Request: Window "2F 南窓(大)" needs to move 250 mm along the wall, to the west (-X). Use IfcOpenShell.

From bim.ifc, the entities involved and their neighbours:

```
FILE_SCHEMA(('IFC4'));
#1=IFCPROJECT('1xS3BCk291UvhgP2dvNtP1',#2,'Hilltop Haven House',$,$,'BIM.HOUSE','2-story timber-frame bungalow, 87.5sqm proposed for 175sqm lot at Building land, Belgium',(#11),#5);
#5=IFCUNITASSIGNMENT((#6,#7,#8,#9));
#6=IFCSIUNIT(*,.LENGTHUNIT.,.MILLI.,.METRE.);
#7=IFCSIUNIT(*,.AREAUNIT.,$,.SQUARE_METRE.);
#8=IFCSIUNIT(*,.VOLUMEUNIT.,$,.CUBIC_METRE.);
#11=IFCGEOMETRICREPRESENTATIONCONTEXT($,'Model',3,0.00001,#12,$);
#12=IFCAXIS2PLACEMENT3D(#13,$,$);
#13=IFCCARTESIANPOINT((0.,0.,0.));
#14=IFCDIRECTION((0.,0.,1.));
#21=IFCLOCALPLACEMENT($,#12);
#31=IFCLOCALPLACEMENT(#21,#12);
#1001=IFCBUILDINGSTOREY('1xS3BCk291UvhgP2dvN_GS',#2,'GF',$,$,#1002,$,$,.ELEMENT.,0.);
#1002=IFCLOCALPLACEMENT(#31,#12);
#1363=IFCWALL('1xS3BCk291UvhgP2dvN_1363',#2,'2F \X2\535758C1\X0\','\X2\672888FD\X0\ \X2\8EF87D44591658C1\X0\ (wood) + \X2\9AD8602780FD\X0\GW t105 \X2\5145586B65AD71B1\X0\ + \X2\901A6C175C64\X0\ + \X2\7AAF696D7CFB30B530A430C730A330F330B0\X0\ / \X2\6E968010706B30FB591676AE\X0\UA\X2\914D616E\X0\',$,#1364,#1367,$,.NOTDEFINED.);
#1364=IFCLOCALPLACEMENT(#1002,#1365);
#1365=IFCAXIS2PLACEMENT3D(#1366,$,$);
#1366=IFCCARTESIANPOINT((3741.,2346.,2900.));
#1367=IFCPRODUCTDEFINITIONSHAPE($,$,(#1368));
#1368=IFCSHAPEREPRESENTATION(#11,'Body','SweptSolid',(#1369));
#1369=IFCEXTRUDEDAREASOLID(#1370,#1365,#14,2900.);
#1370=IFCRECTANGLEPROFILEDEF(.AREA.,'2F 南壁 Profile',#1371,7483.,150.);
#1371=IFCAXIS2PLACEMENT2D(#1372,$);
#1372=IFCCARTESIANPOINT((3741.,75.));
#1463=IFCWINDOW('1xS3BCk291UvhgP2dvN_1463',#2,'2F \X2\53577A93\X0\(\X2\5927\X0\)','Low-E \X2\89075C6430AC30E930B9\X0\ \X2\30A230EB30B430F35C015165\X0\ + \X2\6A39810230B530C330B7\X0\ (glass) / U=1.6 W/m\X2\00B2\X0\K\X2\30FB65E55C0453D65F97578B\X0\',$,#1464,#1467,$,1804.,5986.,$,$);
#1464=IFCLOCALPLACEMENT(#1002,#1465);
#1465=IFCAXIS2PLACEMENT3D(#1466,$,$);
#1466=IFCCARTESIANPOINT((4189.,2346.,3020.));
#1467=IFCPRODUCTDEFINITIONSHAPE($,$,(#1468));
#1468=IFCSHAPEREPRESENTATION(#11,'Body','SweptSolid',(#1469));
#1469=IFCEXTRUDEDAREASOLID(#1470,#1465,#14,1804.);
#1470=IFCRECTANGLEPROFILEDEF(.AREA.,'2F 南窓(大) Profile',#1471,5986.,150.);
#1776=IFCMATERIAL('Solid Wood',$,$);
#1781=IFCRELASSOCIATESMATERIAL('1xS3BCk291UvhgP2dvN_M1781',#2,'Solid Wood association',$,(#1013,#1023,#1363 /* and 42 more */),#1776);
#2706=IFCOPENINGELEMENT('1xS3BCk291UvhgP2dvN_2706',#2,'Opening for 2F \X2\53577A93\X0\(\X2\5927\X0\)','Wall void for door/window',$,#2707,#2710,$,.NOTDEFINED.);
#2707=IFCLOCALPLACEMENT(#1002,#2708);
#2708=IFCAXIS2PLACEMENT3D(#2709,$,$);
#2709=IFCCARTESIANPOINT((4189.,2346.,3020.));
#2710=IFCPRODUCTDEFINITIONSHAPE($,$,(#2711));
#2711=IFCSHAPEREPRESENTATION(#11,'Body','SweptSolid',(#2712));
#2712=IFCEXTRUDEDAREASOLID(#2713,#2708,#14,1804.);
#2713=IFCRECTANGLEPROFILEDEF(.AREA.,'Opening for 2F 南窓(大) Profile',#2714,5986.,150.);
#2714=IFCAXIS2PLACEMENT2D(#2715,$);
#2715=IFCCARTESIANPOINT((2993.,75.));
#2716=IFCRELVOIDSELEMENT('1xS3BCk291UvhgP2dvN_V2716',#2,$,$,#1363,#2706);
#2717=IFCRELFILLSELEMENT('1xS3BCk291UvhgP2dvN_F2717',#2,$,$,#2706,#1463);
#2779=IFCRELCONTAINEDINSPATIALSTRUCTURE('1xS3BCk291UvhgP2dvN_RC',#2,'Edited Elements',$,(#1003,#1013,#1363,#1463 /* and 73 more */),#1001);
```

```python
import ifcopenshell
import ifcopenshell.api.geometry
import ifcopenshell.util.placement
import ifcopenshell.util.unit

model = ifcopenshell.open("bim.ifc")
unit_scale = ifcopenshell.util.unit.calculate_unit_scale(model)

window = model.by_guid("1xS3BCk291UvhgP2dvN_1463")
opening = window.FillsVoids[0].RelatingOpeningElement
wall = opening.VoidsElements[0].RelatingBuildingElement

wall_matrix = ifcopenshell.util.placement.get_local_placement(wall.ObjectPlacement)
shift = wall_matrix[:3, 0] * -0.25 / unit_scale
before = ifcopenshell.util.placement.get_local_placement(window.ObjectPlacement)[:3, 3].copy()

# The window is not placed relative to its opening, so move both.
for product in (opening, window):
    matrix = ifcopenshell.util.placement.get_local_placement(product.ObjectPlacement)
    matrix[:3, 3] += shift
    ifcopenshell.api.geometry.edit_object_placement(model, product=product, matrix=matrix, is_si=False)

after = ifcopenshell.util.placement.get_local_placement(window.ObjectPlacement)[:3, 3]
print("window moved by", (after - before).round(3) + 0.0)

model.write("bim_edited.ifc")
```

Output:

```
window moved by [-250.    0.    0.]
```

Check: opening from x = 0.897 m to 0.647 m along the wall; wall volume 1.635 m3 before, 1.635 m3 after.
